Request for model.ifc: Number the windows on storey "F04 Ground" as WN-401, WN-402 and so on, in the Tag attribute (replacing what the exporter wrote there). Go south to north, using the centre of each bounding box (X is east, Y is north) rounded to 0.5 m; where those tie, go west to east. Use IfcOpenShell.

First a look at what the model holds.

```python
import ifcopenshell
import ifcopenshell.util.element
import ifcopenshell.util.placement

model = ifcopenshell.open("model.ifc")
print(model.schema)
storey = next(s for s in model.by_type("IfcBuildingStorey") if s.Name == "F04 Ground")
windows = [e for e in ifcopenshell.util.element.get_decomposition(storey) if e.is_a("IfcWindow")]
for e in sorted(windows, key=lambda e: e.id()):
    origin = ifcopenshell.util.placement.get_local_placement(e.ObjectPlacement)[:3, 3]
    print(e.id(), e.Tag, e.Name, origin.round(2) + 0.0, sep=" | ")
```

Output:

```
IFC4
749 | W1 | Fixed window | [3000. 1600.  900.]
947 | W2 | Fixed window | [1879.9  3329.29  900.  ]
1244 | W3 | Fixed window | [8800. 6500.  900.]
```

```python
import ifcopenshell
import ifcopenshell.geom
import ifcopenshell.util.element
import ifcopenshell.util.shape

model = ifcopenshell.open("model.ifc")
settings = ifcopenshell.geom.settings()
settings.set("use-world-coords", True)


def centre(element):
    shape = ifcopenshell.geom.create_shape(settings, element)
    return ifcopenshell.util.shape.get_bbox_centroid(shape.geometry)


storey = next(s for s in model.by_type("IfcBuildingStorey") if s.Name == "F04 Ground")
windows = [e for e in ifcopenshell.util.element.get_decomposition(storey) if e.is_a("IfcWindow")]

# Insertion points can sit at a corner or the storey origin, so sort by the geometry (in metres).
centres = {e: centre(e) for e in windows}
windows.sort(key=lambda e: (round(centres[e][1] / 0.5), centres[e][0]))

for i, e in enumerate(windows, start=1):
    number = f"WN-4{i:02d}"
    e.Tag = number
    print(e.id(), number)

model.write("model_edited.ifc")
```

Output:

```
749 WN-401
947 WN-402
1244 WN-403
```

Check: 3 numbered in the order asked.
